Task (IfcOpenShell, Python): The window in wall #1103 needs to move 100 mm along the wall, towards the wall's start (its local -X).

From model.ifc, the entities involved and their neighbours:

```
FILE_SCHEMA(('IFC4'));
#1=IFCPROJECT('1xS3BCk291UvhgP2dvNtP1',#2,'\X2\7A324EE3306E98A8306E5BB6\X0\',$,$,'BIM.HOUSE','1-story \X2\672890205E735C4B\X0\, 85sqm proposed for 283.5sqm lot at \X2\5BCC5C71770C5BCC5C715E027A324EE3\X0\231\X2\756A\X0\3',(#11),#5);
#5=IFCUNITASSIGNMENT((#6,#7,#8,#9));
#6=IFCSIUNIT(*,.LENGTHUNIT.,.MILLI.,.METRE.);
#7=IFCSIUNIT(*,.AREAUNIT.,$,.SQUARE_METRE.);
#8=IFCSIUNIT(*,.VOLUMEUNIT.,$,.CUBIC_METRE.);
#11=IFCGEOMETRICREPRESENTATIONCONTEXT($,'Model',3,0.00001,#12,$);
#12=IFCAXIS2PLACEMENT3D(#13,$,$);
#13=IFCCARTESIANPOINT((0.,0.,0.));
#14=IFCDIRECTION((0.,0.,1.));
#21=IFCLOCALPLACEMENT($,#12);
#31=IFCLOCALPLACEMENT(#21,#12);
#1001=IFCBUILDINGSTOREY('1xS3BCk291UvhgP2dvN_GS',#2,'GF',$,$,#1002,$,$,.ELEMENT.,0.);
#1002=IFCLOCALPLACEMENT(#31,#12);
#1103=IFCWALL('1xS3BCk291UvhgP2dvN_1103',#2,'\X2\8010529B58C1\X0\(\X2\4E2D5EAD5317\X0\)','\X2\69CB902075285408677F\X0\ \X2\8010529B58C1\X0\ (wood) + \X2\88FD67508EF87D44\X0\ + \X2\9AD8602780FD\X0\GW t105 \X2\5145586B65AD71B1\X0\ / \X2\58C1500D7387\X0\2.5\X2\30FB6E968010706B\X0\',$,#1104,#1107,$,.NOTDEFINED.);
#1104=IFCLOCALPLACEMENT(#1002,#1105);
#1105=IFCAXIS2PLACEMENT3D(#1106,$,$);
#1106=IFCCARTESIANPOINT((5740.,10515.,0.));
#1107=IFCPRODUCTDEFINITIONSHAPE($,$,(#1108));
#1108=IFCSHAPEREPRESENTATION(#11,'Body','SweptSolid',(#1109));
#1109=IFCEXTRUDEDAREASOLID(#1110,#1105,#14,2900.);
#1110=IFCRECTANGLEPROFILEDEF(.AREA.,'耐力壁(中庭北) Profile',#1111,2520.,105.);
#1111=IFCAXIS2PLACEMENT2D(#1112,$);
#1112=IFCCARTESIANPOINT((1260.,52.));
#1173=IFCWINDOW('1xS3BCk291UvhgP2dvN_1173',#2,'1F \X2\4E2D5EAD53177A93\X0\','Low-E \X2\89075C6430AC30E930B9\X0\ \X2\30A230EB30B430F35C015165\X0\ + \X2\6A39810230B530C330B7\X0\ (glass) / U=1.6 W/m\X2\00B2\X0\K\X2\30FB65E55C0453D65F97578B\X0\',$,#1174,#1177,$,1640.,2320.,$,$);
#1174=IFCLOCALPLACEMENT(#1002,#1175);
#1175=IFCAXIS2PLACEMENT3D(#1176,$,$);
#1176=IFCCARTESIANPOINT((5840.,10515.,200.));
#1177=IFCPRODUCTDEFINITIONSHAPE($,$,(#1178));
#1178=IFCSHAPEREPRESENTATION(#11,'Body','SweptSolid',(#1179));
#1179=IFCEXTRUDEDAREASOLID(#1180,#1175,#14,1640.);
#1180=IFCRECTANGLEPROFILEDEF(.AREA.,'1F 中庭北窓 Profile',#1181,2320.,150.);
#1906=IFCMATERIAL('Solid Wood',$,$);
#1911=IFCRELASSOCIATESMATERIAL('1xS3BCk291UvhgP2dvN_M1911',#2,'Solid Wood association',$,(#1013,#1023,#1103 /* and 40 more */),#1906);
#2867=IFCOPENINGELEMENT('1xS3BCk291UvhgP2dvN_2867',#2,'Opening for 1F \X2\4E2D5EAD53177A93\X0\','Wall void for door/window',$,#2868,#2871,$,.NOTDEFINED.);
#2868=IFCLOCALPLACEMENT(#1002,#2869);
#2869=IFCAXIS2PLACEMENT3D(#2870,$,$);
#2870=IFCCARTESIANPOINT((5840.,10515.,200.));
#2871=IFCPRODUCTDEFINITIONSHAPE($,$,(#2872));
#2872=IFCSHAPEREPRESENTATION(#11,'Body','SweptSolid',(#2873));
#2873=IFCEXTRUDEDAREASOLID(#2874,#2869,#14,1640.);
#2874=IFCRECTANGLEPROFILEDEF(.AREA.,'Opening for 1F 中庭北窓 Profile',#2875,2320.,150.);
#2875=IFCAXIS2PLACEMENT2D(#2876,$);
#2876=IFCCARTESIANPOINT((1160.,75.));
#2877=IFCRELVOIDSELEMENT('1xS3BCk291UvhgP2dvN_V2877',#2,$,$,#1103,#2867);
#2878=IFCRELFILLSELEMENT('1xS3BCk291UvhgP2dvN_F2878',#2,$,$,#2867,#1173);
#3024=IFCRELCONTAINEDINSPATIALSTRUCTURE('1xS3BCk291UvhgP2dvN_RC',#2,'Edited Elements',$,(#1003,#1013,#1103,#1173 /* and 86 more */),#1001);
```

```python
import ifcopenshell
import ifcopenshell.api.geometry
import ifcopenshell.util.placement
import ifcopenshell.util.unit

model = ifcopenshell.open("model.ifc")
unit_scale = ifcopenshell.util.unit.calculate_unit_scale(model)

window = model.by_id(1173)
opening = window.FillsVoids[0].RelatingOpeningElement
wall = opening.VoidsElements[0].RelatingBuildingElement

wall_matrix = ifcopenshell.util.placement.get_local_placement(wall.ObjectPlacement)
shift = wall_matrix[:3, 0] * -0.1 / unit_scale
before = ifcopenshell.util.placement.get_local_placement(window.ObjectPlacement)[:3, 3].copy()

# The window is not placed relative to its opening, so move both.
for product in (opening, window):
    matrix = ifcopenshell.util.placement.get_local_placement(product.ObjectPlacement)
    matrix[:3, 3] += shift
    ifcopenshell.api.geometry.edit_object_placement(model, product=product, matrix=matrix, is_si=False)

after = ifcopenshell.util.placement.get_local_placement(window.ObjectPlacement)[:3, 3]
print("window moved by", (after - before).round(3) + 0.0)

model.write("model-out.ifc")
```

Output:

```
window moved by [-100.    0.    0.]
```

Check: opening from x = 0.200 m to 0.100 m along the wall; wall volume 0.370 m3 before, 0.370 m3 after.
